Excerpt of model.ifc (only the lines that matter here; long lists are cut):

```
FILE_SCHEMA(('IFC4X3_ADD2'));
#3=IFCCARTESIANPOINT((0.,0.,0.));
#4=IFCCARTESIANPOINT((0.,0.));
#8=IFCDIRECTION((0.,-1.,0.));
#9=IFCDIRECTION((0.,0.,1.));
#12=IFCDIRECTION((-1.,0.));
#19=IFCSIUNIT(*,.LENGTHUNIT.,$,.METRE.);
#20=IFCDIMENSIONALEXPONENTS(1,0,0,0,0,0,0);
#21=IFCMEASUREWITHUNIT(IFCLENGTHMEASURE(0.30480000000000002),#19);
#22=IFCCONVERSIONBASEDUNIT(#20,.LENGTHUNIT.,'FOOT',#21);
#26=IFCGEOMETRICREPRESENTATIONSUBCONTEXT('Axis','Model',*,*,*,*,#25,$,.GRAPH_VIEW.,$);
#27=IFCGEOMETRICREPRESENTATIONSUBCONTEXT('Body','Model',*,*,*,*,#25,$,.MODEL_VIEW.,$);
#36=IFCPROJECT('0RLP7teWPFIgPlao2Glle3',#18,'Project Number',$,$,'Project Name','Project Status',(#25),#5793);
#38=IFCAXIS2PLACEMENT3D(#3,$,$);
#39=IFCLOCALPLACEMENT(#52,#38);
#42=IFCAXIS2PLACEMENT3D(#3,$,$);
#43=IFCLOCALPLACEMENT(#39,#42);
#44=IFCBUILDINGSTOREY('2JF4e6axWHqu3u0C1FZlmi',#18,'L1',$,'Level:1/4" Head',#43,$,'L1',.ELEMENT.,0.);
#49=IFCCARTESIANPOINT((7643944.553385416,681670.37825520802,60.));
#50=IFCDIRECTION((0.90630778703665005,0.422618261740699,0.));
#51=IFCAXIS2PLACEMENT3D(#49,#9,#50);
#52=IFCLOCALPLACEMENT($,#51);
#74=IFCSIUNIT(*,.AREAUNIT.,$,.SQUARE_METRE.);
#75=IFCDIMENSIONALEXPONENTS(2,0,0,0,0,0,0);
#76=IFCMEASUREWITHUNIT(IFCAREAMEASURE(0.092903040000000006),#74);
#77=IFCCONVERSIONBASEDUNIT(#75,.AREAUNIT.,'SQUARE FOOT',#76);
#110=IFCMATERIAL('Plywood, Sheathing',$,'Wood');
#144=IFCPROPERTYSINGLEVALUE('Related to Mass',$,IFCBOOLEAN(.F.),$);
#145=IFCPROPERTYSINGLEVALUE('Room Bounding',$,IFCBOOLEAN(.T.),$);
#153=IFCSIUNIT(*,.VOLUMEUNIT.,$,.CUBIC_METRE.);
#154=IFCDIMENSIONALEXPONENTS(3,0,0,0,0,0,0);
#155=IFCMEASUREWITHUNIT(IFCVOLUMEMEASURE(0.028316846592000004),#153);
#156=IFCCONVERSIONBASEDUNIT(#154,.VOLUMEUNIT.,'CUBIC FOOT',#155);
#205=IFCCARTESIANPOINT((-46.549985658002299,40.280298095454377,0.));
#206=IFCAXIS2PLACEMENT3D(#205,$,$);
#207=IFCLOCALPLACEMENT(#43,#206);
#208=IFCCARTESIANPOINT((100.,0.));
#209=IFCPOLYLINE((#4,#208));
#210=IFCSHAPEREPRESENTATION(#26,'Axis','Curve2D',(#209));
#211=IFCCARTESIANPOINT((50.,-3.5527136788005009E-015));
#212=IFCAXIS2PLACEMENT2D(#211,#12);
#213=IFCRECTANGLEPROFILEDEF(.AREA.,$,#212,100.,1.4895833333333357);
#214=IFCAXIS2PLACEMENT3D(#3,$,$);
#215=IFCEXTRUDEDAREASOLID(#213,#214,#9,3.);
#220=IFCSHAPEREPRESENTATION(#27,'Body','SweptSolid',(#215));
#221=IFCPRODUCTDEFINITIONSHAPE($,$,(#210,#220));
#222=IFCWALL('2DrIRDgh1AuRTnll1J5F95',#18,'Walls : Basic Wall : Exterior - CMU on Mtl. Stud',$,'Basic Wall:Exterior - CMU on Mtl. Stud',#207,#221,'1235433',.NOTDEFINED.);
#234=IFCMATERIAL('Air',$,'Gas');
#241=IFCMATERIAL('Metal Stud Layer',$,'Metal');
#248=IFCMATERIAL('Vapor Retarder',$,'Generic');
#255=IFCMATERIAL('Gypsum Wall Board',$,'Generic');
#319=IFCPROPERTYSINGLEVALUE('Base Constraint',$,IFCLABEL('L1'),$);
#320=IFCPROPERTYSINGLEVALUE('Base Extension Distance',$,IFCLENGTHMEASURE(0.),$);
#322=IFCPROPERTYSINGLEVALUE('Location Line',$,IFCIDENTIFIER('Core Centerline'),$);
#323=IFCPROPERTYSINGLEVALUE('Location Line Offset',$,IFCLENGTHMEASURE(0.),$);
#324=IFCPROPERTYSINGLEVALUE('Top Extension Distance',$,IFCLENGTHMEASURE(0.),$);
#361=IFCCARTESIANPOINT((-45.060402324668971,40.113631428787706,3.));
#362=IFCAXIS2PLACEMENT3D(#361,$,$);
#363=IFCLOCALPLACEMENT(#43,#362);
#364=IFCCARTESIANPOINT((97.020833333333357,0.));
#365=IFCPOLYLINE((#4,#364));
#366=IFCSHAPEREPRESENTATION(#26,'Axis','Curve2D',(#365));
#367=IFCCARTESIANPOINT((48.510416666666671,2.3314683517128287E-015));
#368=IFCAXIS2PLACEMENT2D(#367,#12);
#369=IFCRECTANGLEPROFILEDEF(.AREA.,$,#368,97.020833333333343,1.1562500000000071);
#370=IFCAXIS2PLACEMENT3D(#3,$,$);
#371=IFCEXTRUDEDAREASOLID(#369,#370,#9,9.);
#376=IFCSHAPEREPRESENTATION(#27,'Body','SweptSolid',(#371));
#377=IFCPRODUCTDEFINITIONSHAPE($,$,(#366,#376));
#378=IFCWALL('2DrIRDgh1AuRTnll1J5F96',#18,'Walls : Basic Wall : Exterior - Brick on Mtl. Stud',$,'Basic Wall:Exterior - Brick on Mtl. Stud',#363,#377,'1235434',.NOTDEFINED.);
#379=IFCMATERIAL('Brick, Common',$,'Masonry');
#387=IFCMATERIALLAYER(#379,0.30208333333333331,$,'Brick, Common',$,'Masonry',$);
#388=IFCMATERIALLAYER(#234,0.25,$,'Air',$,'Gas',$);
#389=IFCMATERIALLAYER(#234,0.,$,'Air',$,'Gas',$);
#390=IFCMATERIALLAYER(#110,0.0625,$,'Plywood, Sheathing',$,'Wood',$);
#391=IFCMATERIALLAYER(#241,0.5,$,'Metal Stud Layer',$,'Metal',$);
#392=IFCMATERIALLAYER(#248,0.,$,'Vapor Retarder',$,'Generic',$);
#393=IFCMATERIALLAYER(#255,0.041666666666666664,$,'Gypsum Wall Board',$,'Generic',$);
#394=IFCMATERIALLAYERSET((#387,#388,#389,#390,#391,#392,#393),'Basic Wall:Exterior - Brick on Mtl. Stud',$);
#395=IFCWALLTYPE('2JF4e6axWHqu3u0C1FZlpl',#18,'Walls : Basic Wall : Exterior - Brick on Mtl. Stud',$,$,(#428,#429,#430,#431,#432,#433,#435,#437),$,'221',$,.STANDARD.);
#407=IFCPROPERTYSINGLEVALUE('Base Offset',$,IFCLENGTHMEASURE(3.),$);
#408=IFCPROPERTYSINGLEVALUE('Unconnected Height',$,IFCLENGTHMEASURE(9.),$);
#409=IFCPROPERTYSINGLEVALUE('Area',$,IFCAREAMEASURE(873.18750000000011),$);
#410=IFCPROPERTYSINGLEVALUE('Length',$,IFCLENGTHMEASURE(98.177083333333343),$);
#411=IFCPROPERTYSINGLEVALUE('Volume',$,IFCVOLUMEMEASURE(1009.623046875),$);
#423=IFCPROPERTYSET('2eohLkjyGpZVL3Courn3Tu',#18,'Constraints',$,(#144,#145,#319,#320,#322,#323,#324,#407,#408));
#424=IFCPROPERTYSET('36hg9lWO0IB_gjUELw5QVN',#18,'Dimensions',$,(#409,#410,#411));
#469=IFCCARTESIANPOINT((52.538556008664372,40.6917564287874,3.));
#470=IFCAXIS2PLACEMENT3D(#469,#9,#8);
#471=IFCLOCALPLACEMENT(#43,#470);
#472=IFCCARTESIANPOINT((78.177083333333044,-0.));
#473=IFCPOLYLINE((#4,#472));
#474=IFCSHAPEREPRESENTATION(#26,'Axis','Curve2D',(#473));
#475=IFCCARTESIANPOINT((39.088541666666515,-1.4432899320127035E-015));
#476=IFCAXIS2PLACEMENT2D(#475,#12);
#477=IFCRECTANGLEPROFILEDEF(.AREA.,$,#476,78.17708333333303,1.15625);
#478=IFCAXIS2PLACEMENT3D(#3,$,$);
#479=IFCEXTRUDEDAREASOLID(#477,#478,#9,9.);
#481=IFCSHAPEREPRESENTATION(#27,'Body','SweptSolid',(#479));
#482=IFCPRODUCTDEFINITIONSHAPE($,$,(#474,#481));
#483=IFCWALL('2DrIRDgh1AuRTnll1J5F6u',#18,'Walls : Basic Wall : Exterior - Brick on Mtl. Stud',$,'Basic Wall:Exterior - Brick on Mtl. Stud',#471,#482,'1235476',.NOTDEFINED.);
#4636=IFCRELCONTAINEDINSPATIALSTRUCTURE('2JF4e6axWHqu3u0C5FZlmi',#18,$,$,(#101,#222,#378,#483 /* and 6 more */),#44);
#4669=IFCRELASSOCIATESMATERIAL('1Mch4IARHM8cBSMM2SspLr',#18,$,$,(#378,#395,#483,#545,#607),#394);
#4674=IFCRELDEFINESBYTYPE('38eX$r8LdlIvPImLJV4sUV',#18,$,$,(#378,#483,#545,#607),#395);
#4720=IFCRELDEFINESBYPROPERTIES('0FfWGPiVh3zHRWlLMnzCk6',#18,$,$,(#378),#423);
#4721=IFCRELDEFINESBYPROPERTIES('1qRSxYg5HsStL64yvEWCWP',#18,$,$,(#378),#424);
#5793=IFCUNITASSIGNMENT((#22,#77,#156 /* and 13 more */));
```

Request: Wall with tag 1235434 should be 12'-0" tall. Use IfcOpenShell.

```python
import ifcopenshell
import ifcopenshell.api.pset
import ifcopenshell.geom
import ifcopenshell.util.element
import ifcopenshell.util.representation
import ifcopenshell.util.shape
import ifcopenshell.util.unit

model = ifcopenshell.open("model.ifc")
unit_scale = ifcopenshell.util.unit.calculate_unit_scale(model)
area_scale = ifcopenshell.util.unit.calculate_unit_scale(model, "AREAUNIT")
volume_scale = ifcopenshell.util.unit.calculate_unit_scale(model, "VOLUMEUNIT")
settings = ifcopenshell.geom.settings()


def volume(element):
    """Net volume in cubic metres, openings subtracted."""
    shape = ifcopenshell.geom.create_shape(settings, element)
    return ifcopenshell.util.shape.get_volume(shape.geometry)


wall = model.by_guid("2DrIRDgh1AuRTnll1J5F96")
before = volume(wall)

body = ifcopenshell.util.representation.get_representation(wall, "Model", "Body")
solid = body.Items[0]
old_height = solid.Depth
solid.Depth = 144 * 0.0254 / unit_scale
after = volume(wall)
thickness = 0.3524  # wall thickness in metres

# Update the stored height, areas and volumes.
pset = model.by_id(ifcopenshell.util.element.get_pset(wall, "Constraints", should_inherit=False)["id"])
ifcopenshell.api.pset.edit_pset(model, pset=pset, properties={
    "Unconnected Height": model.create_entity("IfcLengthMeasure", solid.Depth),
})
pset = model.by_id(ifcopenshell.util.element.get_pset(wall, "Dimensions", should_inherit=False)["id"])
ifcopenshell.api.pset.edit_pset(model, pset=pset, properties={
    "Area": model.create_entity("IfcAreaMeasure", after / thickness / area_scale),
    "Volume": model.create_entity("IfcVolumeMeasure", after / volume_scale),
})

print(f"height {old_height:g} -> {solid.Depth:g}, volume {before:.3f} -> {after:.3f} m3")

model.write("model_updated.ifc")
```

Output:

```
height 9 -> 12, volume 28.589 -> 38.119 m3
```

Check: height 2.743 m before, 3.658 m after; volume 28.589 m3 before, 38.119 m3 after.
